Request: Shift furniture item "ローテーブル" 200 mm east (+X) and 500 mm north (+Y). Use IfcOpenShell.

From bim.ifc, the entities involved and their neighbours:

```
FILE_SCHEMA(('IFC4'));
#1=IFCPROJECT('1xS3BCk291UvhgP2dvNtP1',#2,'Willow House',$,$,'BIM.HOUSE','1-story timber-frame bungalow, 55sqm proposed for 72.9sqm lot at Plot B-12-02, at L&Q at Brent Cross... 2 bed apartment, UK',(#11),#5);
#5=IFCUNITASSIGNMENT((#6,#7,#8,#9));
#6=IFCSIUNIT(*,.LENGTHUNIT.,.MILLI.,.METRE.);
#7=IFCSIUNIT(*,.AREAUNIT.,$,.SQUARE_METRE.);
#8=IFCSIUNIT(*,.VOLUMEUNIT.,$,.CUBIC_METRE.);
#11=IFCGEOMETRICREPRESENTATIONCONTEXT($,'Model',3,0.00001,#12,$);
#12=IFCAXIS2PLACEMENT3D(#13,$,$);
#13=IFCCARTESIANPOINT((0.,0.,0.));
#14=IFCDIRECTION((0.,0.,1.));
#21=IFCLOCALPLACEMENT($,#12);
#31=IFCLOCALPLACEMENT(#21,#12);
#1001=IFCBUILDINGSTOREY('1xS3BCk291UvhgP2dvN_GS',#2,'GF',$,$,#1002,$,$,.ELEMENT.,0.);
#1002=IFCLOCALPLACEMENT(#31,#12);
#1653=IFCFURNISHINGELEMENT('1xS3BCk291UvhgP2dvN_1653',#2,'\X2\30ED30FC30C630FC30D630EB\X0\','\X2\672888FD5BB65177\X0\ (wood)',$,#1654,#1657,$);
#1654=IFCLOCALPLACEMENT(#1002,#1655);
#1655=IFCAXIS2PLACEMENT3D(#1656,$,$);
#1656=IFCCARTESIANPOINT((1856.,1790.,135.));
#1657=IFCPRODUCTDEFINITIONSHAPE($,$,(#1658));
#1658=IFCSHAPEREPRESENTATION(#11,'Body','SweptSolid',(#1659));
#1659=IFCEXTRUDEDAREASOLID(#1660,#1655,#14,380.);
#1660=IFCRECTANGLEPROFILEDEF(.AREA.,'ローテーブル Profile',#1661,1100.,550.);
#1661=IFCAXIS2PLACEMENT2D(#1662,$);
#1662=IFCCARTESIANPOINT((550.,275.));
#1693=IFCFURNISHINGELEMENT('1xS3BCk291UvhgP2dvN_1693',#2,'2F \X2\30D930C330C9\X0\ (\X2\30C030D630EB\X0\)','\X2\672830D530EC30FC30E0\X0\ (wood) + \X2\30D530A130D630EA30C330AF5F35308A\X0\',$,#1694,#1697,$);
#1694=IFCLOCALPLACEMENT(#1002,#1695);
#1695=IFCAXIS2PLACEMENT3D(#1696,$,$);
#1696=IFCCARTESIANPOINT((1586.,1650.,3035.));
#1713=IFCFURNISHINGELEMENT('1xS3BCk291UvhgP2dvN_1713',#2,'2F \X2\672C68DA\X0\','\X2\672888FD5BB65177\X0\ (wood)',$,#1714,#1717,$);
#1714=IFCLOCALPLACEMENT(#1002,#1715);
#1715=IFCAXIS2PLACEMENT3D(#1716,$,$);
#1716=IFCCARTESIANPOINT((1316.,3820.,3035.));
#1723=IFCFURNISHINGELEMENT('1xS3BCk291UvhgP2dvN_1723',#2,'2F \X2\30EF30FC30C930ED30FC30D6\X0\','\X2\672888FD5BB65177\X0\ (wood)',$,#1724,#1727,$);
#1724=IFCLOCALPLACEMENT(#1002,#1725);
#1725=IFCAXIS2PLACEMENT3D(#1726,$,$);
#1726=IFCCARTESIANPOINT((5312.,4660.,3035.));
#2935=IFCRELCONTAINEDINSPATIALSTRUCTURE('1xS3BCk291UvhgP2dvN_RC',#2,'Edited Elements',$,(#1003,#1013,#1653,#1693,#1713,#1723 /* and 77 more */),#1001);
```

```python
import ifcopenshell
import ifcopenshell.api.geometry
import ifcopenshell.util.placement
import ifcopenshell.util.unit

model = ifcopenshell.open("bim.ifc")
unit_scale = ifcopenshell.util.unit.calculate_unit_scale(model)

item = model.by_guid("1xS3BCk291UvhgP2dvN_1653")
matrix = ifcopenshell.util.placement.get_local_placement(item.ObjectPlacement)
matrix[0, 3] += 0.2 / unit_scale
matrix[1, 3] += 0.5 / unit_scale
ifcopenshell.api.geometry.edit_object_placement(model, product=item, matrix=matrix, is_si=False)

print(ifcopenshell.util.placement.get_local_placement(item.ObjectPlacement).round(3) + 0.0)

model.write("bim_v2.ifc")
```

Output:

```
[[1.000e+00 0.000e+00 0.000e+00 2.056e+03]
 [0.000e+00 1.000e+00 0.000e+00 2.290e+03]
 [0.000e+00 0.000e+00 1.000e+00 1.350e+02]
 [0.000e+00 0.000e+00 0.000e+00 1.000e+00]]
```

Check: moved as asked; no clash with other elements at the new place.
